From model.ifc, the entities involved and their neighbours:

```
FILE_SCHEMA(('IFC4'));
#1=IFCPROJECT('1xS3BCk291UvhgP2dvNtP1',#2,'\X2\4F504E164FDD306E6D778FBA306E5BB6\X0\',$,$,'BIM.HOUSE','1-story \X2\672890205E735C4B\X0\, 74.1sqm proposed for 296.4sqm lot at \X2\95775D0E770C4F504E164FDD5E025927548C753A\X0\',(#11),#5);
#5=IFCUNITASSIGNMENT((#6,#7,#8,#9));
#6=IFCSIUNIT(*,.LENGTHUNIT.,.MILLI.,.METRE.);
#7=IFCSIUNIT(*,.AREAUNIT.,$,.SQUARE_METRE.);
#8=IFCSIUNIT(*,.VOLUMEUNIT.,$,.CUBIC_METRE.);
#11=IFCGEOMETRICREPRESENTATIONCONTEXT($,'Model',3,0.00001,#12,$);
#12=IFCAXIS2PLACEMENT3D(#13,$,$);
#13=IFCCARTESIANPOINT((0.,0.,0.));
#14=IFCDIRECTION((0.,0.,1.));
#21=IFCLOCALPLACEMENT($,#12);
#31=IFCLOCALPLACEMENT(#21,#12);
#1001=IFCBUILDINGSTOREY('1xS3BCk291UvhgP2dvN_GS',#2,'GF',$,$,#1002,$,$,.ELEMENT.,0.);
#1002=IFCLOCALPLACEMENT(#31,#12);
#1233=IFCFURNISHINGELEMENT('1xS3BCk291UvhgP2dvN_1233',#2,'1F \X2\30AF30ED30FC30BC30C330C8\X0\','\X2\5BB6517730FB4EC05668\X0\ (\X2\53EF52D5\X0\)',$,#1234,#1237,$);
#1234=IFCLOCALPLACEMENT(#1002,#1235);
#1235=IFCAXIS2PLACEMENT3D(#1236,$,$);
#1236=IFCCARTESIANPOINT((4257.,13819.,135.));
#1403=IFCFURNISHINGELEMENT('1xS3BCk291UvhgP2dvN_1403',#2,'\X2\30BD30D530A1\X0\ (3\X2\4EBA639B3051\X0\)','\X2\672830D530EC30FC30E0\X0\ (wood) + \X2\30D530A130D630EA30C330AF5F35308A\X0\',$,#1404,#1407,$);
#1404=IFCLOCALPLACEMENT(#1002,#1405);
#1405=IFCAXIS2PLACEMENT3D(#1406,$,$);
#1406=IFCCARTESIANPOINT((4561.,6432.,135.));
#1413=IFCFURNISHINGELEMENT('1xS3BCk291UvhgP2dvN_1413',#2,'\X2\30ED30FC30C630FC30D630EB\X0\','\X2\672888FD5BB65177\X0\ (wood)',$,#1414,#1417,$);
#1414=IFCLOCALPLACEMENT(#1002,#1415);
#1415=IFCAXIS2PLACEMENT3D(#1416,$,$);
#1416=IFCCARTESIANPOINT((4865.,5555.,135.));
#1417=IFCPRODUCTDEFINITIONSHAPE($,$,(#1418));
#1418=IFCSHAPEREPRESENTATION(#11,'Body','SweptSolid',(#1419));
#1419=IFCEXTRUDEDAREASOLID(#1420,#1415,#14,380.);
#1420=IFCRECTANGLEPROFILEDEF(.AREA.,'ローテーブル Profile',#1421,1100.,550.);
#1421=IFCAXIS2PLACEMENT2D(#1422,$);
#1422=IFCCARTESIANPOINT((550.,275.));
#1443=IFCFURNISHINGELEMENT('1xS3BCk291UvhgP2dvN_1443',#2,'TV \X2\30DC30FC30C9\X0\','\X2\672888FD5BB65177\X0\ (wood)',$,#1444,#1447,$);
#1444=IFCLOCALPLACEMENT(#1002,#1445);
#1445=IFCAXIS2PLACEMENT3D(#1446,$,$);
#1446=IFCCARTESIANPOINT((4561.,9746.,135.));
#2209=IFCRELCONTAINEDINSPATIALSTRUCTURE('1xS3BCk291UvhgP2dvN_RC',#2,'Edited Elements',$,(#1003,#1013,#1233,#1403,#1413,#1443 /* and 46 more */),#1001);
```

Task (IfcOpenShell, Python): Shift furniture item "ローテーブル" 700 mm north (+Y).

```python
import ifcopenshell
import ifcopenshell.api.geometry
import ifcopenshell.util.placement
import ifcopenshell.util.unit

model = ifcopenshell.open("model.ifc")
unit_scale = ifcopenshell.util.unit.calculate_unit_scale(model)

item = model.by_id(1413)
matrix = ifcopenshell.util.placement.get_local_placement(item.ObjectPlacement)
matrix[1, 3] += 0.7 / unit_scale
ifcopenshell.api.geometry.edit_object_placement(model, product=item, matrix=matrix, is_si=False)

print(ifcopenshell.util.placement.get_local_placement(item.ObjectPlacement).round(3) + 0.0)

model.write("model_edited.ifc")
```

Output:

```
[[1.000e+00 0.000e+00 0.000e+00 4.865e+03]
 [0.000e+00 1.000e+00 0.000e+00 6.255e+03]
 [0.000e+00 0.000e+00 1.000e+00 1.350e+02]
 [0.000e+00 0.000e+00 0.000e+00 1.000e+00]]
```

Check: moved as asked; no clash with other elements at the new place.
